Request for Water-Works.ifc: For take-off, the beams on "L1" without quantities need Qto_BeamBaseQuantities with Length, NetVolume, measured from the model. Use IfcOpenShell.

First a look at what the model holds.

```python
import ifcopenshell
import ifcopenshell.util.element
import ifcopenshell.util.unit

model = ifcopenshell.open("Water-Works.ifc")
print(model.schema)
for unit_type in ("LENGTHUNIT", "AREAUNIT", "VOLUMEUNIT"):
    print(unit_type, ifcopenshell.util.unit.calculate_unit_scale(model, unit_type))
storey = next(s for s in model.by_type("IfcBuildingStorey") if s.Name == "L1")
beams = [e for e in ifcopenshell.util.element.get_decomposition(storey) if e.is_a("IfcBeam")]
for e in sorted(beams, key=lambda e: e.id()):
    print(e.id(), e.is_a(), e.Name, list(ifcopenshell.util.element.get_psets(e, qtos_only=True)), sep=" | ")
```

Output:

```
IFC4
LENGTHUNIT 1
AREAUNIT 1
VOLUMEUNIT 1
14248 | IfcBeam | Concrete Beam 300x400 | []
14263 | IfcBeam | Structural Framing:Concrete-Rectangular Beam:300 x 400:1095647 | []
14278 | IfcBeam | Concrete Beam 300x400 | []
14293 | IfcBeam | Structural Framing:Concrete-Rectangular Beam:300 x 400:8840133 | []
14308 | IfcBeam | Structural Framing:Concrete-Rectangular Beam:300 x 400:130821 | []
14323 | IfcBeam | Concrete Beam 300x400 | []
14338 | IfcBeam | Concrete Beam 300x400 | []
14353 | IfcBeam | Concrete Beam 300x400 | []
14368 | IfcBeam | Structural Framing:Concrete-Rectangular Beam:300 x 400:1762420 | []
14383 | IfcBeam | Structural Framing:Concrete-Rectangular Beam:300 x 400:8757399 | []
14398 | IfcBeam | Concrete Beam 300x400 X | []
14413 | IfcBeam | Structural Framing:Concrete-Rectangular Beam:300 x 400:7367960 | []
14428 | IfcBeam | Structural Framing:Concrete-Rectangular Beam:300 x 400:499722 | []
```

```python
import ifcopenshell
import ifcopenshell.api.pset
import ifcopenshell.geom
import ifcopenshell.util.element
import ifcopenshell.util.shape
import ifcopenshell.util.unit

model = ifcopenshell.open("Water-Works.ifc")
unit_scale = ifcopenshell.util.unit.calculate_unit_scale(model)
volume_scale = ifcopenshell.util.unit.calculate_unit_scale(model, "VOLUMEUNIT")
settings = ifcopenshell.geom.settings()

storey = next(s for s in model.by_type("IfcBuildingStorey") if s.Name == "L1")
beams = [e for e in ifcopenshell.util.element.get_decomposition(storey) if e.is_a("IfcBeam")]

for e in sorted(beams, key=lambda e: e.id()):
    if ifcopenshell.util.element.get_psets(e, qtos_only=True, should_inherit=False):
        continue
    # Geometry comes back in metres, in the element's own axes.
    shape = ifcopenshell.geom.create_shape(settings, e)
    values = {
        "Length": ifcopenshell.util.shape.get_max_xyz(shape.geometry) / unit_scale,
        "NetVolume": ifcopenshell.util.shape.get_volume(shape.geometry) / volume_scale,
    }
    qto = ifcopenshell.api.pset.add_qto(model, product=e, name="Qto_BeamBaseQuantities")
    ifcopenshell.api.pset.edit_qto(model, qto=qto, properties=values)
    print(e.id(), {k: round(v, 3) for k, v in values.items()})

model.write("Water-Works-out.ifc")
```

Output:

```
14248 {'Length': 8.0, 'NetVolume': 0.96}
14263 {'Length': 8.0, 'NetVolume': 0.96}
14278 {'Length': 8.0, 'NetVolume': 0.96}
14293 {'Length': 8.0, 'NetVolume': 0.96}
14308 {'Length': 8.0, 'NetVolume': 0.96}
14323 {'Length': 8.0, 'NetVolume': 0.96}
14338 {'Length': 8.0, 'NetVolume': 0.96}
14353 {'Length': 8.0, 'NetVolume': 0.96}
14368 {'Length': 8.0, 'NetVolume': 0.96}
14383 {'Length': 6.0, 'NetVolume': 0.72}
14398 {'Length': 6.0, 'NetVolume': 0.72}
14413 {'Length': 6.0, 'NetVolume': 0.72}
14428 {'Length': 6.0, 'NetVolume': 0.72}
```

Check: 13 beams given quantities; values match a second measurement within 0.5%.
